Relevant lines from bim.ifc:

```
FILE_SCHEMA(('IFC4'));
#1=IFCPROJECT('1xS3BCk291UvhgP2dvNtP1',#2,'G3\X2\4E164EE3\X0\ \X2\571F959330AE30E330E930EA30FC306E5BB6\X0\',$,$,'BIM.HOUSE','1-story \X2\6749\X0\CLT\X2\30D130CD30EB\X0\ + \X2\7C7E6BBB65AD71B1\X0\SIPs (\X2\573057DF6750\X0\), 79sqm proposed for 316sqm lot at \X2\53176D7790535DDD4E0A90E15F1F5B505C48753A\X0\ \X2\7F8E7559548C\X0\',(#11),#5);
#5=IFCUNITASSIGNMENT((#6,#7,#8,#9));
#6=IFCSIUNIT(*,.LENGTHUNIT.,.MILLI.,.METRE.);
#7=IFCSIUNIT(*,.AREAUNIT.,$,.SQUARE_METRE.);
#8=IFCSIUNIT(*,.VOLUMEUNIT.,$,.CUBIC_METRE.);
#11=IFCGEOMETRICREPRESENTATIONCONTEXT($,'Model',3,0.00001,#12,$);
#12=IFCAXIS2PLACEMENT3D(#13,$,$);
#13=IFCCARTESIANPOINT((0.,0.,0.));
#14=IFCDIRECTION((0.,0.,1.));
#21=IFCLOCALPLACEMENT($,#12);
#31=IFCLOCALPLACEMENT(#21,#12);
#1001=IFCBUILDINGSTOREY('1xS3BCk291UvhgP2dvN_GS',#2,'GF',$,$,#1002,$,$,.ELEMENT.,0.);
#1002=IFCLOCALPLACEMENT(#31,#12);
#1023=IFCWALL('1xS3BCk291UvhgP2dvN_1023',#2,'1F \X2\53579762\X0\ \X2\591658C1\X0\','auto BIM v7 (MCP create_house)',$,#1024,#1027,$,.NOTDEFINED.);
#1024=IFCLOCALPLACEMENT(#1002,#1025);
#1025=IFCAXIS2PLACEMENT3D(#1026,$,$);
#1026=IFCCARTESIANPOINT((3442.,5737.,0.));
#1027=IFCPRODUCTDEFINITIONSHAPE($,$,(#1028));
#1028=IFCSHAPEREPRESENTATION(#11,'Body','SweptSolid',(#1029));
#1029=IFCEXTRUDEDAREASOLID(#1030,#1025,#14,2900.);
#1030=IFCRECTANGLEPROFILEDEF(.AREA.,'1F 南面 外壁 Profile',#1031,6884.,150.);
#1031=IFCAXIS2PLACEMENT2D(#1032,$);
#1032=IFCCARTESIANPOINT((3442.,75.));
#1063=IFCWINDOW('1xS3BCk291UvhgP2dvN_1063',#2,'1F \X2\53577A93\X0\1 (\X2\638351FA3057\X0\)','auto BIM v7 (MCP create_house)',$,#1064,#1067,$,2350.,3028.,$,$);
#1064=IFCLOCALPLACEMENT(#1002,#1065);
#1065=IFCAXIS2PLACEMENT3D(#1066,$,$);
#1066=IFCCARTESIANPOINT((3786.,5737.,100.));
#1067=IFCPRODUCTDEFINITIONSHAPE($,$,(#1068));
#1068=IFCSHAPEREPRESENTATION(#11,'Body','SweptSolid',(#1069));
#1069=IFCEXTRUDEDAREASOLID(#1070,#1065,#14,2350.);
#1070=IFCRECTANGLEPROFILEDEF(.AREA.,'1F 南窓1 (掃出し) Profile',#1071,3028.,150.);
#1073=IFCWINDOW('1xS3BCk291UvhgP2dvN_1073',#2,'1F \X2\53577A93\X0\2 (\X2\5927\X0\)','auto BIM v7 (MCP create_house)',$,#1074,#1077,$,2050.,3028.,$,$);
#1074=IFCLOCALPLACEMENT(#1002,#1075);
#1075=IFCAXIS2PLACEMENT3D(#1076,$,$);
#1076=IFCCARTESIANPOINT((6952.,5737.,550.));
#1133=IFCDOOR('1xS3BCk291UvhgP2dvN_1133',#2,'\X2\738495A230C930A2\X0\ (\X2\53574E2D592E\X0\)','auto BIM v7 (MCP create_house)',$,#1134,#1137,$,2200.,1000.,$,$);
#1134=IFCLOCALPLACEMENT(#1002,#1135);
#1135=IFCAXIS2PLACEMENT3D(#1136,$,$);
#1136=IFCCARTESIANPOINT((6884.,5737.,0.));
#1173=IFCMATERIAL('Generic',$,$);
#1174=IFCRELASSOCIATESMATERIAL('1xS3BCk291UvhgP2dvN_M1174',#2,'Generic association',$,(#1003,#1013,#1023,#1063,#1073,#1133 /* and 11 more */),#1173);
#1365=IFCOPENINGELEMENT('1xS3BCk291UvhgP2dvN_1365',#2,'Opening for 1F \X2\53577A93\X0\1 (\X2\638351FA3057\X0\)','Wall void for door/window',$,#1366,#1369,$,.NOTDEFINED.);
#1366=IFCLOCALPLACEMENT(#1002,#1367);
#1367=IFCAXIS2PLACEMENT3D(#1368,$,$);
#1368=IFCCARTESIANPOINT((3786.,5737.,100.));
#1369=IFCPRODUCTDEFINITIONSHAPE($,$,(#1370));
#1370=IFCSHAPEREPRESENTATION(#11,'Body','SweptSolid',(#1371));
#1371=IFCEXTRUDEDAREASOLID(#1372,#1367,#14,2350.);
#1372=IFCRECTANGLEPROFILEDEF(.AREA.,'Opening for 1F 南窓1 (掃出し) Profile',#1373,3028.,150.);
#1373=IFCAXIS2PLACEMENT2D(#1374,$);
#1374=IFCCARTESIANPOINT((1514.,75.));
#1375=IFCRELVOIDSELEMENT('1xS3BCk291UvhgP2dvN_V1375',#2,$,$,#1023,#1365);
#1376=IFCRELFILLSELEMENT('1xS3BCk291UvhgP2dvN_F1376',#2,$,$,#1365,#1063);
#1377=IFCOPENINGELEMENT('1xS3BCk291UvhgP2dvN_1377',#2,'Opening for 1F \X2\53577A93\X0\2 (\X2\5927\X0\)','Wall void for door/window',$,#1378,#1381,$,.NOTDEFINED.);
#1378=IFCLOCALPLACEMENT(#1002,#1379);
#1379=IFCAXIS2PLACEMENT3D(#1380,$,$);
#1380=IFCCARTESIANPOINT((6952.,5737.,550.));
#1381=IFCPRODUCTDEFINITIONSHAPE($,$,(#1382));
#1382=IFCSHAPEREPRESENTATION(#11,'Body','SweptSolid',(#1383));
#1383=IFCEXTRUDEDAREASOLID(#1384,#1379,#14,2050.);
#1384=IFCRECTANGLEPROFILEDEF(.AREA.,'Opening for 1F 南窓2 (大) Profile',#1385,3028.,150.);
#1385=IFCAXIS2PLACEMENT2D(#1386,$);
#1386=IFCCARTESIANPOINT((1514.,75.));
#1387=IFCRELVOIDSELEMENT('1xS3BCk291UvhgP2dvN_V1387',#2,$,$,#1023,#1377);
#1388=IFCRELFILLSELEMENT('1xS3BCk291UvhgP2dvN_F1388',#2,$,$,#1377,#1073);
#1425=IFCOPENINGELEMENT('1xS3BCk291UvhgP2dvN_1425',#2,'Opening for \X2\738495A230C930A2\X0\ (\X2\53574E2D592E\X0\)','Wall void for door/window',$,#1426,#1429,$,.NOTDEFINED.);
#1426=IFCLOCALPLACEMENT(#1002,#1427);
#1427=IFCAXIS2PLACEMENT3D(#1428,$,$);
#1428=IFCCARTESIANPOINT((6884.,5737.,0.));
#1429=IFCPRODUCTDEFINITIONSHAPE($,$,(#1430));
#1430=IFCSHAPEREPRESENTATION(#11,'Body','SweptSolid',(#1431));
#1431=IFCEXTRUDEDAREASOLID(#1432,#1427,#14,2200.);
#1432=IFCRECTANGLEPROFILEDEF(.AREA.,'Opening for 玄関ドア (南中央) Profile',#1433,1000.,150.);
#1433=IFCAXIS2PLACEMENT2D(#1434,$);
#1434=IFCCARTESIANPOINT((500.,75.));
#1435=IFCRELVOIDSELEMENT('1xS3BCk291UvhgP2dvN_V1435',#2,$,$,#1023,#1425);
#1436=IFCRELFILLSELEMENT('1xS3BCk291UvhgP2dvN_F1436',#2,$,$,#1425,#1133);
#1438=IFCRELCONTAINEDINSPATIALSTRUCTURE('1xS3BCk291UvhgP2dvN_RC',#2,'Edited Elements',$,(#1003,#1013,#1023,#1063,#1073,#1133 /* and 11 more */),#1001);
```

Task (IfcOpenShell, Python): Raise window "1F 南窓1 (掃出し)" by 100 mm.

```python
import numpy as np
import ifcopenshell
import ifcopenshell.api.geometry
import ifcopenshell.util.placement
import ifcopenshell.util.unit

model = ifcopenshell.open("bim.ifc")
unit_scale = ifcopenshell.util.unit.calculate_unit_scale(model)

window = model.by_guid("1xS3BCk291UvhgP2dvN_1063")
opening = window.FillsVoids[0].RelatingOpeningElement
dz = 100.0

shift = np.array([0.0, 0.0, dz])
# The window is not placed relative to its opening, so move both.
for product in (opening, window):
    matrix = ifcopenshell.util.placement.get_local_placement(product.ObjectPlacement)
    matrix[:3, 3] += shift
    ifcopenshell.api.geometry.edit_object_placement(model, product=product, matrix=matrix, is_si=False)

print(f"moved by {dz * unit_scale:+.3f} m")

model.write("bim_edited.ifc")
```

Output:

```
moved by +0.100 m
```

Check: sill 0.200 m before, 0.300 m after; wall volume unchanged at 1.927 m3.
